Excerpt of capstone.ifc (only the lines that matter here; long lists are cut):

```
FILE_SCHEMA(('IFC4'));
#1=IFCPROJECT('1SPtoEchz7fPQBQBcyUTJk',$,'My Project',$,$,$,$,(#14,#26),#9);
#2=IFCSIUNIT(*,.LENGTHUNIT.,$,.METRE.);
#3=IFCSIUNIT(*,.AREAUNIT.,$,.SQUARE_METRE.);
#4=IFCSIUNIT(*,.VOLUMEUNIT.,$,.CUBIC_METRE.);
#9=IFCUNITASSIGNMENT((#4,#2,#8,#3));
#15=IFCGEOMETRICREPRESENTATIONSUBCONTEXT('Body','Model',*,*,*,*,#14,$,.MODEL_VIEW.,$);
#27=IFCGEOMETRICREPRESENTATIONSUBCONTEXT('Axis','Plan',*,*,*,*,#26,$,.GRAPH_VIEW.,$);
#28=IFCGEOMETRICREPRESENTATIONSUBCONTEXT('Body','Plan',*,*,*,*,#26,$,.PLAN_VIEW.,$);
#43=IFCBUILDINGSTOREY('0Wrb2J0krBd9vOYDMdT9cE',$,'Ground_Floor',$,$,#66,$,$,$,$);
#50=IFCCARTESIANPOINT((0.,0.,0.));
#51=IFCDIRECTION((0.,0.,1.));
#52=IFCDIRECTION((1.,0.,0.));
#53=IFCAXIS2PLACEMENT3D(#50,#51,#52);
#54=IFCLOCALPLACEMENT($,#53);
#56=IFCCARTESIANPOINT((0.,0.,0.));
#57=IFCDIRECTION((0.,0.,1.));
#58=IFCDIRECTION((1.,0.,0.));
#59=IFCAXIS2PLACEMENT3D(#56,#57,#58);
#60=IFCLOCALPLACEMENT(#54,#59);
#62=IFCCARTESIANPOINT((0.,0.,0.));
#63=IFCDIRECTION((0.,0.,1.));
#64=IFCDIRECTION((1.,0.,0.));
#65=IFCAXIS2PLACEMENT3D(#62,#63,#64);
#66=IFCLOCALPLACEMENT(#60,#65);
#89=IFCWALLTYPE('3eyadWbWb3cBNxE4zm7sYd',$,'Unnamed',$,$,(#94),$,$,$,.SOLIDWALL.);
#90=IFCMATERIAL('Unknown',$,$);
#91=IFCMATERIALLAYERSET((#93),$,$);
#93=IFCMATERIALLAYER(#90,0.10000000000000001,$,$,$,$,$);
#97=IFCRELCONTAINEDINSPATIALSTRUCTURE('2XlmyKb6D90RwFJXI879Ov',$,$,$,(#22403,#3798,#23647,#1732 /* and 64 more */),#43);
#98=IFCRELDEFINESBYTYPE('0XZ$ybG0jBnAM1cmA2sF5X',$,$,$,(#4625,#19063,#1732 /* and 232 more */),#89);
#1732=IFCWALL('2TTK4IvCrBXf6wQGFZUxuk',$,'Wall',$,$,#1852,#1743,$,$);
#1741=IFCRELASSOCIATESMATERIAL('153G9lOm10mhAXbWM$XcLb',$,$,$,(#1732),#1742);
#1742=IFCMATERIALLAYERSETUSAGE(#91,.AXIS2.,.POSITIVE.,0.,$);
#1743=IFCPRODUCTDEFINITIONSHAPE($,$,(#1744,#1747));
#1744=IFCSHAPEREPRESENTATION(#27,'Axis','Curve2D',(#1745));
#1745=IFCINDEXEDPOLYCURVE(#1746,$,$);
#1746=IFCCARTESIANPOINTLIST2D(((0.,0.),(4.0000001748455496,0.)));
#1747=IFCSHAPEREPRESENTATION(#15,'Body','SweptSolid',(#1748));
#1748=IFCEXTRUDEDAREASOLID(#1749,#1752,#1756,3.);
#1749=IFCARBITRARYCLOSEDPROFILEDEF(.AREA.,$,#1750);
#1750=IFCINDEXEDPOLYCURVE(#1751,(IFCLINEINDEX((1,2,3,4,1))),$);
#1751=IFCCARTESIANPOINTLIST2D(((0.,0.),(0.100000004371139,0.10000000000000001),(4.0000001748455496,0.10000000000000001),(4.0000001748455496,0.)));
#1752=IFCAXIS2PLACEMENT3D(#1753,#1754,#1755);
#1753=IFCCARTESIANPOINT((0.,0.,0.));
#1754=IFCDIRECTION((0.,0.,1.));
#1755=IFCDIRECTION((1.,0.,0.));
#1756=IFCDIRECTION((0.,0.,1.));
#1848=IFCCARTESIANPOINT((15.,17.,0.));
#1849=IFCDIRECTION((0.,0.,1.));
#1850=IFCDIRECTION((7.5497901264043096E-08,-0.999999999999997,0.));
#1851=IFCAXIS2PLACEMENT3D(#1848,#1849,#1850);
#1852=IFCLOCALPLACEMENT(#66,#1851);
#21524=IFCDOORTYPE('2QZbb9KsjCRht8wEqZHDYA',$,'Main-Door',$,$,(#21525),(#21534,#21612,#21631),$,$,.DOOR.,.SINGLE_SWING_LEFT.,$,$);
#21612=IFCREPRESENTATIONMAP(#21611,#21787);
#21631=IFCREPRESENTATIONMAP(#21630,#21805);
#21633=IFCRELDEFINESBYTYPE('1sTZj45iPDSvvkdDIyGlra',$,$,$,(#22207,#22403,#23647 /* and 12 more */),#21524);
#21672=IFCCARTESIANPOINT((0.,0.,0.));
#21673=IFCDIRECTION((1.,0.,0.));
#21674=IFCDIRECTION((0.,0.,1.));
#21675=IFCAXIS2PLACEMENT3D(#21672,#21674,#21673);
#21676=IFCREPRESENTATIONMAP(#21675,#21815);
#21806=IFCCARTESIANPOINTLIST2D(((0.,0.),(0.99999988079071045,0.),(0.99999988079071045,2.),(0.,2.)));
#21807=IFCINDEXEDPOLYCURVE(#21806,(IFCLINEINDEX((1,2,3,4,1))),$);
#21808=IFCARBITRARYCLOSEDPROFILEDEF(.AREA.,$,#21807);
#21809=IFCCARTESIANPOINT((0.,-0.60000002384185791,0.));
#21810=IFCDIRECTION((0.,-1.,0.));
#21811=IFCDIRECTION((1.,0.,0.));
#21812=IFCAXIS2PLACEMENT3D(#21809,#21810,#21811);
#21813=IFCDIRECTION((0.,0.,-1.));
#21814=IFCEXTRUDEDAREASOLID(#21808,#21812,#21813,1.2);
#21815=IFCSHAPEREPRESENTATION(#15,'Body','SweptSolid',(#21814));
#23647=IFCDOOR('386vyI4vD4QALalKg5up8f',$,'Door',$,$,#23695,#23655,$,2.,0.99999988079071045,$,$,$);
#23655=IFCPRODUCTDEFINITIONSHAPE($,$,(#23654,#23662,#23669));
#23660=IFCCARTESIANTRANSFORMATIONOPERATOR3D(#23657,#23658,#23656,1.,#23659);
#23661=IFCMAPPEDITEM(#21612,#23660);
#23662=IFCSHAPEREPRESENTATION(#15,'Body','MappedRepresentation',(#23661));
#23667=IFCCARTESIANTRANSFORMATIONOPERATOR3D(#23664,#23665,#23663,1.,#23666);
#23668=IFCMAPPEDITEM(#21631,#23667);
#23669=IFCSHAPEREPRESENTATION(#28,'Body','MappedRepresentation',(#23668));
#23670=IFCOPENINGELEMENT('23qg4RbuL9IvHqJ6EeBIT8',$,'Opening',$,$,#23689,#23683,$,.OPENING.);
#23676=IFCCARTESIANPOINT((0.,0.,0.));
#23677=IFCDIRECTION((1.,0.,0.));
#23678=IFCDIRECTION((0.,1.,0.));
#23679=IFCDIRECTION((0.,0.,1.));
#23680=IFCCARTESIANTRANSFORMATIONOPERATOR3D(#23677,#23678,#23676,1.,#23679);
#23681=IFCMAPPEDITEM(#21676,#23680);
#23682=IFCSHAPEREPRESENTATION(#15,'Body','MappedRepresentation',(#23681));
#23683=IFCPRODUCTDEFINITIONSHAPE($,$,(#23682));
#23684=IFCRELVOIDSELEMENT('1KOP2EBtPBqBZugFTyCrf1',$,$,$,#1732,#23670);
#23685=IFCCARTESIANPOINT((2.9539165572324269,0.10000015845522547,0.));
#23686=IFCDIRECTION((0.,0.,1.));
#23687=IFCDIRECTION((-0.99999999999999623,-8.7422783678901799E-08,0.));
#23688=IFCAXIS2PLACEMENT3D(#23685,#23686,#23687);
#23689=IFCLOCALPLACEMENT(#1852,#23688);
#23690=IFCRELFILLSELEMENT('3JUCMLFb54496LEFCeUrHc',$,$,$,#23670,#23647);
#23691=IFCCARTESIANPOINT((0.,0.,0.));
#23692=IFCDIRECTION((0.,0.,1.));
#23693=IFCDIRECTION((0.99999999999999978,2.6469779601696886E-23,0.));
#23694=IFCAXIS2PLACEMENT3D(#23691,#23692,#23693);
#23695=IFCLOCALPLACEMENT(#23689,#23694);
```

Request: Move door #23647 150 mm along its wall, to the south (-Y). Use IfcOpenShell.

```python
import ifcopenshell
import ifcopenshell.api.geometry
import ifcopenshell.util.placement
import ifcopenshell.util.unit

model = ifcopenshell.open("capstone.ifc")
unit_scale = ifcopenshell.util.unit.calculate_unit_scale(model)

door = model.by_id(23647)
opening = door.FillsVoids[0].RelatingOpeningElement
wall = opening.VoidsElements[0].RelatingBuildingElement

wall_matrix = ifcopenshell.util.placement.get_local_placement(wall.ObjectPlacement)
shift = wall_matrix[:3, 0] * 0.15 / unit_scale
before = ifcopenshell.util.placement.get_local_placement(door.ObjectPlacement)[:3, 3].copy()

# The door is placed relative to its opening, so it follows when the opening moves.
matrix = ifcopenshell.util.placement.get_local_placement(opening.ObjectPlacement)
matrix[:3, 3] += shift
ifcopenshell.api.geometry.edit_object_placement(
    model, product=opening, matrix=matrix, is_si=False, should_transform_children=True
)

after = ifcopenshell.util.placement.get_local_placement(door.ObjectPlacement)[:3, 3]
print("door moved by", (after - before).round(3) + 0.0)

model.write("capstone-out.ifc")
```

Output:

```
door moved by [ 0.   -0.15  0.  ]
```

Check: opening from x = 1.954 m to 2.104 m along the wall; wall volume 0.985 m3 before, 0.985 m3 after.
